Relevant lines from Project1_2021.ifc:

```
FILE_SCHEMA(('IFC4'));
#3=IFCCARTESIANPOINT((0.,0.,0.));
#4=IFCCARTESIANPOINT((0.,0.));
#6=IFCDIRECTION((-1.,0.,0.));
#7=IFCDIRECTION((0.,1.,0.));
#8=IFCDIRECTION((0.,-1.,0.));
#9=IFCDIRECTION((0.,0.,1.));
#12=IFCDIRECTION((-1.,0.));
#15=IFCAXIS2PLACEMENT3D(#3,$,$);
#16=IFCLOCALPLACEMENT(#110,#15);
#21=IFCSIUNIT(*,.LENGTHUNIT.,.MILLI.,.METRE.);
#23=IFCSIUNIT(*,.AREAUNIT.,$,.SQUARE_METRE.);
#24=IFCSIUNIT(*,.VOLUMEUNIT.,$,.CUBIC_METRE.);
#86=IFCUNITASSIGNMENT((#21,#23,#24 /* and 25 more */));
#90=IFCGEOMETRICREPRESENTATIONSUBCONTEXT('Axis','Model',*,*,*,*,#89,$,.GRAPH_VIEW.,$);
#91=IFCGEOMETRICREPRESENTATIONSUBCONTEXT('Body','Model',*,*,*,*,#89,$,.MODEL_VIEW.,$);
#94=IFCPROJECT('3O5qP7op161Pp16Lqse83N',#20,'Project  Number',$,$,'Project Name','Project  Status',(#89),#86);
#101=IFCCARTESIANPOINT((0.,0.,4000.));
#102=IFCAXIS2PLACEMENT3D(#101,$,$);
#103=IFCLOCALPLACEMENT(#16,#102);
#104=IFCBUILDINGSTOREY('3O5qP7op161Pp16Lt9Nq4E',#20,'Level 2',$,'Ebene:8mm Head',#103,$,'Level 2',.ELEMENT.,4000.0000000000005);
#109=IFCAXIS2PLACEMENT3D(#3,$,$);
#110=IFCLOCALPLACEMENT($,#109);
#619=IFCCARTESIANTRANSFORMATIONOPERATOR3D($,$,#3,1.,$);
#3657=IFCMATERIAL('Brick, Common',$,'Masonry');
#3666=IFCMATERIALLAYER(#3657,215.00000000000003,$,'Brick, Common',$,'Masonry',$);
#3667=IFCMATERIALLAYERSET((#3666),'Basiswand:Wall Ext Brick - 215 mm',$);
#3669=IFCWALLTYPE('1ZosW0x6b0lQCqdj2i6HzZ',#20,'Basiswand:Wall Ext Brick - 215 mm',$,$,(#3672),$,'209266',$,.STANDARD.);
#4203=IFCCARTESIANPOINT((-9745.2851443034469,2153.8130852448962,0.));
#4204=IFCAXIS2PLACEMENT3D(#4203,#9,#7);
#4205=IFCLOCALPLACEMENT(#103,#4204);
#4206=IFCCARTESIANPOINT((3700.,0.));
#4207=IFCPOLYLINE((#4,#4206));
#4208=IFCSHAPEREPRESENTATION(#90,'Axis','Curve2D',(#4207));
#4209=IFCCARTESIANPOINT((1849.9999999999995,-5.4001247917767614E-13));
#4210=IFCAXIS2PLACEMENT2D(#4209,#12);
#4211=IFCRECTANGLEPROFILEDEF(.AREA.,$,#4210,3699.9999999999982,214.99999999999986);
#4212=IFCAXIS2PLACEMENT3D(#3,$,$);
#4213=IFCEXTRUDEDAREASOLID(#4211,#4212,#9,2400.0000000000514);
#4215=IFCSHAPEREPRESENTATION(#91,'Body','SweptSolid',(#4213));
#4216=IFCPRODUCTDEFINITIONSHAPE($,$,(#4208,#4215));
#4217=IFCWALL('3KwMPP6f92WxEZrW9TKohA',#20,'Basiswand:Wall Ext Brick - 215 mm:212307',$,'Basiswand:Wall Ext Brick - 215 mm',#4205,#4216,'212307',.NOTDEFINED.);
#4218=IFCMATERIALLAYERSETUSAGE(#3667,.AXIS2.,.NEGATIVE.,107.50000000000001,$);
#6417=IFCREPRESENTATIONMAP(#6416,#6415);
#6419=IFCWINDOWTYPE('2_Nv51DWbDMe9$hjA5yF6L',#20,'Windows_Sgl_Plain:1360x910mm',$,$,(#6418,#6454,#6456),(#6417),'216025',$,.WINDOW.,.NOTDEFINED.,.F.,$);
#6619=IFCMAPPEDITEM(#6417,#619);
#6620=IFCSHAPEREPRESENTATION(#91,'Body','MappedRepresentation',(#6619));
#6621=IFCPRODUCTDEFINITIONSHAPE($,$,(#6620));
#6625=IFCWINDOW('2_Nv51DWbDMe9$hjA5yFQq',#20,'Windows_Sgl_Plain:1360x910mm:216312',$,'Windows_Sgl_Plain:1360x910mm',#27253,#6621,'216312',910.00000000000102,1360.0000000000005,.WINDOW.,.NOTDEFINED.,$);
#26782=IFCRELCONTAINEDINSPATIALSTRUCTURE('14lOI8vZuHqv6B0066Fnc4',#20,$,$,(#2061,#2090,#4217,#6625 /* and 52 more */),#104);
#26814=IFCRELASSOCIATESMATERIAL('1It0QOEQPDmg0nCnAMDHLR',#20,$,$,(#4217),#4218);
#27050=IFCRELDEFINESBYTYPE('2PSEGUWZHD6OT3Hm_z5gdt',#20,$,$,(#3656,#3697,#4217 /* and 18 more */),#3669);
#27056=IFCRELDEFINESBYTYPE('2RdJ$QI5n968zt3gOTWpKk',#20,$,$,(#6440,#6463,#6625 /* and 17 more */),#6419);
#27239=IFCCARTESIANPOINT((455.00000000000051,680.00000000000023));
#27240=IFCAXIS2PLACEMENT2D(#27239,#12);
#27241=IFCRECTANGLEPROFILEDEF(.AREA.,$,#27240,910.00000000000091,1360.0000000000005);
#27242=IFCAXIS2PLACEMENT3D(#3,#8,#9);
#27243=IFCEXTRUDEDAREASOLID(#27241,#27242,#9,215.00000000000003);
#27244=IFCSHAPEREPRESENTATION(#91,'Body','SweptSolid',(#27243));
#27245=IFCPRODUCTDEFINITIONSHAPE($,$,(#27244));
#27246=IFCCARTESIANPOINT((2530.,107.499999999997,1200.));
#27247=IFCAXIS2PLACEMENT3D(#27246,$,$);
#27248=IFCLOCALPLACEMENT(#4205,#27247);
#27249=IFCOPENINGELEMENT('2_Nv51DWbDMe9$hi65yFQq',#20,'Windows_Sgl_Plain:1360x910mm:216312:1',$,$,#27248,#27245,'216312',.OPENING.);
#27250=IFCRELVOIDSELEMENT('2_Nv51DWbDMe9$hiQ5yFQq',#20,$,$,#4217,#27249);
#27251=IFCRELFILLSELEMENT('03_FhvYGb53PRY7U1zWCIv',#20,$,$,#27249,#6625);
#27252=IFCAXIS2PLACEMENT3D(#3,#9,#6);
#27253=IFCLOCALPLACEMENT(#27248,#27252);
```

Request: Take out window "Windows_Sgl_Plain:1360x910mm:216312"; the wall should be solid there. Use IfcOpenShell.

```python
import ifcopenshell
import ifcopenshell.api.feature
import ifcopenshell.api.root
import ifcopenshell.geom
import ifcopenshell.util.shape

model = ifcopenshell.open("Project1_2021.ifc")
settings = ifcopenshell.geom.settings()


def volume(element):
    """Net volume in cubic metres, openings subtracted."""
    shape = ifcopenshell.geom.create_shape(settings, element)
    return ifcopenshell.util.shape.get_volume(shape.geometry)


window = model.by_guid("2_Nv51DWbDMe9$hjA5yFQq")
opening = window.FillsVoids[0].RelatingOpeningElement
wall = opening.VoidsElements[0].RelatingBuildingElement
before = volume(wall)

ifcopenshell.api.root.remove_product(model, product=window)
ifcopenshell.api.feature.remove_feature(model, feature=opening)

after = volume(wall)

print(f"wall volume {before:.3f} -> {after:.3f} m3")

model.write("Project1_2021_v2.ifc")
```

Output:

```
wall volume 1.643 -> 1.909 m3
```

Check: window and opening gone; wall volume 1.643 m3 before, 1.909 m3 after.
